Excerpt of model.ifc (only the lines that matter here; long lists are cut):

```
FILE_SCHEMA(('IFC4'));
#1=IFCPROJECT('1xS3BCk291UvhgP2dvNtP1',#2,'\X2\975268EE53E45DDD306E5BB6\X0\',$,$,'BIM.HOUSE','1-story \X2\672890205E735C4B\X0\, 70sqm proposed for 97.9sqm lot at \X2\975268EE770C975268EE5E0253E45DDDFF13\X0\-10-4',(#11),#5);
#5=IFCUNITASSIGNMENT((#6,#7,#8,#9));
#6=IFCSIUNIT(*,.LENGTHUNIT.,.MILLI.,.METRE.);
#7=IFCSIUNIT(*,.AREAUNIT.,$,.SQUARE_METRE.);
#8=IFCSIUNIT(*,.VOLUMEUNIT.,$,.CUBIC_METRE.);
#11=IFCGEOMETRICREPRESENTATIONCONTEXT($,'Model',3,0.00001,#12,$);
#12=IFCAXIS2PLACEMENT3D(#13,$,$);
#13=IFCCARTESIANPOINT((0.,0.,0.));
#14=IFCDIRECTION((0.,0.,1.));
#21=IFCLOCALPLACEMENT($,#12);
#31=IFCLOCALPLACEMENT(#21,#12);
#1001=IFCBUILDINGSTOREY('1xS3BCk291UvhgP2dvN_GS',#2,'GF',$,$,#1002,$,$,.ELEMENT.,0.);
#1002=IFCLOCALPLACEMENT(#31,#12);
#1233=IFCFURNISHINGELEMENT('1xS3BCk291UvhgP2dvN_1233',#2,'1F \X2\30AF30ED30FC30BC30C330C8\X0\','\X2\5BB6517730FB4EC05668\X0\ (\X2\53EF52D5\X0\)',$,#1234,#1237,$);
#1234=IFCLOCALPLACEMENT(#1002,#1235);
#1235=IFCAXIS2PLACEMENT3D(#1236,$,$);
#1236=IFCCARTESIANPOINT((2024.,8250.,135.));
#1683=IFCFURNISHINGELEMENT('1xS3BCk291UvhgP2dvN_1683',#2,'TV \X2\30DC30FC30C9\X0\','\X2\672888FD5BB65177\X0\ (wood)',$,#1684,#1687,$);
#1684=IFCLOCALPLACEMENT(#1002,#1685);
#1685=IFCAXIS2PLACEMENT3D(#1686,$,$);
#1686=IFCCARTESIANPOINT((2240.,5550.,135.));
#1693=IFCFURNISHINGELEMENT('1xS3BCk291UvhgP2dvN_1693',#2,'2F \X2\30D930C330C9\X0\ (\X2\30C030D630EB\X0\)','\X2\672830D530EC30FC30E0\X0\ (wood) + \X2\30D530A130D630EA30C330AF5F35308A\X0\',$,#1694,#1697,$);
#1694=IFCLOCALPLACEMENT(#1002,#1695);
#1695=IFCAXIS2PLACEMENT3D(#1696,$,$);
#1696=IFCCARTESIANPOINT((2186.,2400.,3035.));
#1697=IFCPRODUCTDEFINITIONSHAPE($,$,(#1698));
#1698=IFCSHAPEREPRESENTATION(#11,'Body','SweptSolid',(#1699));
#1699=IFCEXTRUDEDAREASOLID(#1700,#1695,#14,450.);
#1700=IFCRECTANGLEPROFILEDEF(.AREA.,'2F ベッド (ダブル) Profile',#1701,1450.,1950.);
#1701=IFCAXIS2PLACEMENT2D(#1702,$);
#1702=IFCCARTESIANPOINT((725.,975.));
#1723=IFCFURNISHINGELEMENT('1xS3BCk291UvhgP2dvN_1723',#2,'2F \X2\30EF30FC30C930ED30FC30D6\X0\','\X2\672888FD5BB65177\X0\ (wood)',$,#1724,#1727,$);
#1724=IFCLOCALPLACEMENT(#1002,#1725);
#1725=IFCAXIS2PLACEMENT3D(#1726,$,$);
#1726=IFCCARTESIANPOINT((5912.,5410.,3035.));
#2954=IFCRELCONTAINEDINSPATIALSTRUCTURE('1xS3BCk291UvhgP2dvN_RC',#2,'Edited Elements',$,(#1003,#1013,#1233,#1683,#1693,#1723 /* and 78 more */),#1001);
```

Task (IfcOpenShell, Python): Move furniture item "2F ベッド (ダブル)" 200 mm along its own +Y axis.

```python
import ifcopenshell
import ifcopenshell.api.geometry
import ifcopenshell.util.placement
import ifcopenshell.util.unit

model = ifcopenshell.open("model.ifc")
unit_scale = ifcopenshell.util.unit.calculate_unit_scale(model)

item = model.by_id(1693)
matrix = ifcopenshell.util.placement.get_local_placement(item.ObjectPlacement)
matrix[:3, 3] += matrix[:3, 1] * 0.2 / unit_scale
ifcopenshell.api.geometry.edit_object_placement(model, product=item, matrix=matrix, is_si=False)

print(ifcopenshell.util.placement.get_local_placement(item.ObjectPlacement).round(3) + 0.0)

model.write("model_rev.ifc")
```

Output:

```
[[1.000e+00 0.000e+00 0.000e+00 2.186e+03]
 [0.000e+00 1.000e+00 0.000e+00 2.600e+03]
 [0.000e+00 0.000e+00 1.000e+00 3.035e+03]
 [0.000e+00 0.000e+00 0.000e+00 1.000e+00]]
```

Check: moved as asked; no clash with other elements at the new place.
